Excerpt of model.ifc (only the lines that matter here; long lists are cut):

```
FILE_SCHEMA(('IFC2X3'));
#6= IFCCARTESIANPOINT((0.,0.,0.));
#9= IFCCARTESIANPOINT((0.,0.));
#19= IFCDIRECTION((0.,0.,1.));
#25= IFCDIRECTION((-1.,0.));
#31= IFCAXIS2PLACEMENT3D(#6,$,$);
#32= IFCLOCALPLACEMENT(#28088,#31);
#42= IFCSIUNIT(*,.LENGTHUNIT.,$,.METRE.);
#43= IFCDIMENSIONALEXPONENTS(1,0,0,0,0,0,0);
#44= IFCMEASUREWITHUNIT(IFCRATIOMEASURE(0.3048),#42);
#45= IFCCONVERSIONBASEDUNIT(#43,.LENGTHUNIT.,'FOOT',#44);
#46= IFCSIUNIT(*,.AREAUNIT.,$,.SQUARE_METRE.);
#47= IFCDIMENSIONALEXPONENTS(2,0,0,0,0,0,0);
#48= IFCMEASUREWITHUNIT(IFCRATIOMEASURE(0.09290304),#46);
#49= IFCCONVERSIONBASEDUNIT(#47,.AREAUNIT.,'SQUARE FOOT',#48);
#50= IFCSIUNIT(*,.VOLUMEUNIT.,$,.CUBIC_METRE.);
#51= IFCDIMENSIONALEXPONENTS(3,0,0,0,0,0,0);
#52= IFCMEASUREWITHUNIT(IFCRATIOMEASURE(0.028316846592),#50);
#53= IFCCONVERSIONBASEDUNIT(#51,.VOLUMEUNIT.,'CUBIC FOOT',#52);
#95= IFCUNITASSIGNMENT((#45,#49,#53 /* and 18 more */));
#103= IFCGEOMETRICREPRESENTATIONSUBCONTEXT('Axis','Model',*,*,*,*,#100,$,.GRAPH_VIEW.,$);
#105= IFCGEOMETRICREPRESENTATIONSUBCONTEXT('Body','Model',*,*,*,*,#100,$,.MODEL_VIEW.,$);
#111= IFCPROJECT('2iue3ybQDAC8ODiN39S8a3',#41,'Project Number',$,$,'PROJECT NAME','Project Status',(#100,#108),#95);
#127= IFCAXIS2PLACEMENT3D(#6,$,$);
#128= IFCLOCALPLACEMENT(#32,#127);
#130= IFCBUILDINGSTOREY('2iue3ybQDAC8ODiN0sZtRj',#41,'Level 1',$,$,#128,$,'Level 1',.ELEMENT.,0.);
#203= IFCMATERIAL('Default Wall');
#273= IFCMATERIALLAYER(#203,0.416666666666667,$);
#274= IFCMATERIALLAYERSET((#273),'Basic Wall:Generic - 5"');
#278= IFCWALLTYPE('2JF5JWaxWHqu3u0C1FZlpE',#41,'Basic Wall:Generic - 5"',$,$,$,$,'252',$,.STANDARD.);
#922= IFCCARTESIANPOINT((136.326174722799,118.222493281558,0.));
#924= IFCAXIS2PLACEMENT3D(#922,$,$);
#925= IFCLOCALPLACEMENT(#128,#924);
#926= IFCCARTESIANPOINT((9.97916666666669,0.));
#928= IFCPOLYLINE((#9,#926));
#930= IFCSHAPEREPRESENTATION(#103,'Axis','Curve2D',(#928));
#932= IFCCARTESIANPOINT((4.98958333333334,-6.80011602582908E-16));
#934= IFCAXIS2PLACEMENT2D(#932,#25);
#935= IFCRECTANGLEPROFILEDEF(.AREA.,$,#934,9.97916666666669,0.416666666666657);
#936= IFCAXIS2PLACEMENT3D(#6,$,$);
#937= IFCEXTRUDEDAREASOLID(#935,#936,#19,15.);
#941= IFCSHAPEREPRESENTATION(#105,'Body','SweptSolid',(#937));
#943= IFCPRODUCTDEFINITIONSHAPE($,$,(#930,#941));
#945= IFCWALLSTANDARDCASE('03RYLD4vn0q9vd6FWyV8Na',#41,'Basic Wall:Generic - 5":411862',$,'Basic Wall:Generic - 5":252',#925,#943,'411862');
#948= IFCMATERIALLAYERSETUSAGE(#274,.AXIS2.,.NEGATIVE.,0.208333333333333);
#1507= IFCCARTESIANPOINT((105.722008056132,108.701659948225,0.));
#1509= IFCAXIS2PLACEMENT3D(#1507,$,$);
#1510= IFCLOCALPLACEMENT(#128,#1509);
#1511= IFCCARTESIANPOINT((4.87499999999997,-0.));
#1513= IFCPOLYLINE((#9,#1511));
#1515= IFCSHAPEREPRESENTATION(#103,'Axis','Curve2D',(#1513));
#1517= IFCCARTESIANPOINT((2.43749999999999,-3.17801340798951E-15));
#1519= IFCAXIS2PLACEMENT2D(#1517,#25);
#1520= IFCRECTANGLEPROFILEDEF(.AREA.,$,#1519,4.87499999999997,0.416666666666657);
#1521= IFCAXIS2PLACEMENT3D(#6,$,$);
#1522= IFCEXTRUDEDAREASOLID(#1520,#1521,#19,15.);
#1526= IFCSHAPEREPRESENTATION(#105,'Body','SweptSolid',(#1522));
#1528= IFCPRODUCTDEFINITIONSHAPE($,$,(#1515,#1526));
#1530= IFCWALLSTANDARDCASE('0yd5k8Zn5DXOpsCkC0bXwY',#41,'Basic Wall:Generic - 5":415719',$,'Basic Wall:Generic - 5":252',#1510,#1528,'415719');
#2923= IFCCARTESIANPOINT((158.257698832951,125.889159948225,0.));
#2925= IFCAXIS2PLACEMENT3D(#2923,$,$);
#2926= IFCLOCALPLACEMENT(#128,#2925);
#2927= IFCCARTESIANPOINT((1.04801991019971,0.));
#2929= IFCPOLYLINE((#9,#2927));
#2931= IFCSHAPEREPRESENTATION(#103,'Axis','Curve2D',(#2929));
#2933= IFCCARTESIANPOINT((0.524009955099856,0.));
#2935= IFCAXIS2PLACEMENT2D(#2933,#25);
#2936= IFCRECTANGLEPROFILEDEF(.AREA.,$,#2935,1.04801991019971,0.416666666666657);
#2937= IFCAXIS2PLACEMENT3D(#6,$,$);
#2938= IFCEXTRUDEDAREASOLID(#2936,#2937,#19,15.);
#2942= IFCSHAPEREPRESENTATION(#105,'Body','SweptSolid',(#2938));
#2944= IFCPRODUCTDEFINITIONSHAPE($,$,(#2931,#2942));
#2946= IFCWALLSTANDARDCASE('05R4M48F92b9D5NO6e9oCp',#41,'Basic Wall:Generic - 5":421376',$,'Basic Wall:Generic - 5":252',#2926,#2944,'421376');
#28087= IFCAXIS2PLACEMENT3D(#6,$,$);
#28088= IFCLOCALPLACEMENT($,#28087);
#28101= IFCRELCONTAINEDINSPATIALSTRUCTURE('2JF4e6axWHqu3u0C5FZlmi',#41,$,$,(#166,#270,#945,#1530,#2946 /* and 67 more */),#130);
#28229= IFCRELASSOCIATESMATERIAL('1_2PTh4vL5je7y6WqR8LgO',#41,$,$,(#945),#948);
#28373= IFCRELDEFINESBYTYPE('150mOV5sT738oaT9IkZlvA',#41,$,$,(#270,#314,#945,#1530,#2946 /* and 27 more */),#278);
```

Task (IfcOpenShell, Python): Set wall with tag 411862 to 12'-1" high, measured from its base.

```python
import ifcopenshell
import ifcopenshell.geom
import ifcopenshell.util.representation
import ifcopenshell.util.shape
import ifcopenshell.util.unit

model = ifcopenshell.open("model.ifc")
unit_scale = ifcopenshell.util.unit.calculate_unit_scale(model)
settings = ifcopenshell.geom.settings()


def volume(element):
    """Net volume in cubic metres, openings subtracted."""
    shape = ifcopenshell.geom.create_shape(settings, element)
    return ifcopenshell.util.shape.get_volume(shape.geometry)


wall = model.by_guid("03RYLD4vn0q9vd6FWyV8Na")
before = volume(wall)

body = ifcopenshell.util.representation.get_representation(wall, "Model", "Body")
solid = body.Items[0]
old_height = solid.Depth
solid.Depth = 145 * 0.0254 / unit_scale
after = volume(wall)

print(f"height {old_height:g} -> {solid.Depth:g}, volume {before:.3f} -> {after:.3f} m3")

model.write("model_v2.ifc")
```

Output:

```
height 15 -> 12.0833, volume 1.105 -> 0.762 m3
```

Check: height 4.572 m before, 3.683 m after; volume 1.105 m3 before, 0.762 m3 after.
